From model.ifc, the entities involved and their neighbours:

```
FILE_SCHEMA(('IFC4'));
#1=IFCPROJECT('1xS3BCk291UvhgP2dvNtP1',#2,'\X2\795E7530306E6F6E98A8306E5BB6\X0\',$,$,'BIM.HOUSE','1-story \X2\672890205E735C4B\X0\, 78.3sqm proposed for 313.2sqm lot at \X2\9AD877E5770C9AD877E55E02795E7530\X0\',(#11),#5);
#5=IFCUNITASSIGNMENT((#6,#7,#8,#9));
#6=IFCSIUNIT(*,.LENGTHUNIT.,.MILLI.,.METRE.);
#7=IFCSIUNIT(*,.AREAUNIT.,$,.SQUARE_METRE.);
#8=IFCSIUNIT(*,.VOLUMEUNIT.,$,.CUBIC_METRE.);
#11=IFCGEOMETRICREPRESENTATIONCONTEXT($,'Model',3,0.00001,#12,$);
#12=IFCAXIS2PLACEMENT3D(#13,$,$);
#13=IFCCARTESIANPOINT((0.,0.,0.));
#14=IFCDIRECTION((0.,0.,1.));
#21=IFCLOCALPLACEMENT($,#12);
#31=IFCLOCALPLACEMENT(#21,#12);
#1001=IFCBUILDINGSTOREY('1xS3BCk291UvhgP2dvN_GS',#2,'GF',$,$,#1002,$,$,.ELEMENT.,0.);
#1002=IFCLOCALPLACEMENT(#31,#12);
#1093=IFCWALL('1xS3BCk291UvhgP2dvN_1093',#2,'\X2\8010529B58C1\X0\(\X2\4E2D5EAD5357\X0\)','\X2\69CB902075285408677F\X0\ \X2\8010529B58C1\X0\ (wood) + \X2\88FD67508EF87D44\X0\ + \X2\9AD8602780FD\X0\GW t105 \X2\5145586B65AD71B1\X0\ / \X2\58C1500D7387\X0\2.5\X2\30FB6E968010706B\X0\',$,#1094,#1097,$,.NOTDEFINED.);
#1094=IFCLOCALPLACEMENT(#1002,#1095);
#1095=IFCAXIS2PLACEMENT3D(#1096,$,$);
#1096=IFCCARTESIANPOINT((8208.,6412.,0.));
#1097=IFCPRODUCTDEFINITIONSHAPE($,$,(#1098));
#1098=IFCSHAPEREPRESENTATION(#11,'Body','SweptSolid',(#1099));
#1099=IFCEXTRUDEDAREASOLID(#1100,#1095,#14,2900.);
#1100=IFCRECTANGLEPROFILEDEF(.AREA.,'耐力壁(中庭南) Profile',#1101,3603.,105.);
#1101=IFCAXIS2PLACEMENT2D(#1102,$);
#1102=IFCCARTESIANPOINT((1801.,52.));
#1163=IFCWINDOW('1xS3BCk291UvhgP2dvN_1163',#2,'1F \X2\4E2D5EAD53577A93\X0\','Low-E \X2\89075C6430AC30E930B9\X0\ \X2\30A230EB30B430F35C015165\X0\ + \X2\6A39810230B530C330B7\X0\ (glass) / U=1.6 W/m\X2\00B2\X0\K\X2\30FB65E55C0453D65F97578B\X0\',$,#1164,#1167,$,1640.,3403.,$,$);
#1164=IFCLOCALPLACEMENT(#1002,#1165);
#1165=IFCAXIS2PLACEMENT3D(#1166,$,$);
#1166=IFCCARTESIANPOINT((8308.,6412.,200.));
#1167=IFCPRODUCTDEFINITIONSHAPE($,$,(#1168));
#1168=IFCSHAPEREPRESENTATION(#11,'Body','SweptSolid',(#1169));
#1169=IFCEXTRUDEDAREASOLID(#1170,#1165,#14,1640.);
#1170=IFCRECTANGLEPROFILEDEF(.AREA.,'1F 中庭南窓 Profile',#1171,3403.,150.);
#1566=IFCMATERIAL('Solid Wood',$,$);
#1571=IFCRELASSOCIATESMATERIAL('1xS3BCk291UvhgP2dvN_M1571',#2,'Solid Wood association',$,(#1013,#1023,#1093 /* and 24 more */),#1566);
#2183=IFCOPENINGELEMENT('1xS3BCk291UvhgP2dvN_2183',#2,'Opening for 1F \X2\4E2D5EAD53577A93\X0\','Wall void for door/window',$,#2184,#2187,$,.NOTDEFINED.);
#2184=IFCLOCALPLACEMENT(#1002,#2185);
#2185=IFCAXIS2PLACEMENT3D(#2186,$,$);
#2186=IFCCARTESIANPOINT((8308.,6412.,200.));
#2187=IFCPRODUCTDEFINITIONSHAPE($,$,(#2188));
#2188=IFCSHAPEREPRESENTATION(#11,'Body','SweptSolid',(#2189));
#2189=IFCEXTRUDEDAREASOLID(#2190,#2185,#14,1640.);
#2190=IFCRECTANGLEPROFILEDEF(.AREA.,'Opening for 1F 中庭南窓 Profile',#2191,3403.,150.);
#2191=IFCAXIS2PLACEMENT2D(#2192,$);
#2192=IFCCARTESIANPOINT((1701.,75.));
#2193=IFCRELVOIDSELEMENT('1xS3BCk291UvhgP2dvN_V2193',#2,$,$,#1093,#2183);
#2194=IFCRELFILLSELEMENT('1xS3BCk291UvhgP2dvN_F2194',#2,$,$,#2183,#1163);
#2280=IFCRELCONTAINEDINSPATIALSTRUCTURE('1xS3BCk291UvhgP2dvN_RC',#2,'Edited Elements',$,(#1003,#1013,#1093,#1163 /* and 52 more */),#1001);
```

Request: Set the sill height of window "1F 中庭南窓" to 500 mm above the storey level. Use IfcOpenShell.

```python
import numpy as np
import ifcopenshell
import ifcopenshell.api.geometry
import ifcopenshell.geom
import ifcopenshell.util.element
import ifcopenshell.util.placement
import ifcopenshell.util.shape
import ifcopenshell.util.unit

model = ifcopenshell.open("model.ifc")
unit_scale = ifcopenshell.util.unit.calculate_unit_scale(model)

window = model.by_guid("1xS3BCk291UvhgP2dvN_1163")
opening = window.FillsVoids[0].RelatingOpeningElement
storey = ifcopenshell.util.element.get_container(window, ifc_class="IfcBuildingStorey")
level = ifcopenshell.util.placement.get_local_placement(storey.ObjectPlacement)[2, 3]

# The opening's origin need not be at the sill, so measure its lowest point.
shape = ifcopenshell.geom.create_shape(ifcopenshell.geom.settings(), opening)
bottom = ifcopenshell.util.shape.get_shape_bottom_elevation(shape, shape.geometry) / unit_scale
dz = level + 500.0 - bottom

shift = np.array([0.0, 0.0, dz])
# The window is not placed relative to its opening, so move both.
for product in (opening, window):
    matrix = ifcopenshell.util.placement.get_local_placement(product.ObjectPlacement)
    matrix[:3, 3] += shift
    ifcopenshell.api.geometry.edit_object_placement(model, product=product, matrix=matrix, is_si=False)

print(f"moved by {dz * unit_scale:+.3f} m")

model.write("model_rev.ifc")
```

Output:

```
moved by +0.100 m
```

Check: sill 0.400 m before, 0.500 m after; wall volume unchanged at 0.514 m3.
